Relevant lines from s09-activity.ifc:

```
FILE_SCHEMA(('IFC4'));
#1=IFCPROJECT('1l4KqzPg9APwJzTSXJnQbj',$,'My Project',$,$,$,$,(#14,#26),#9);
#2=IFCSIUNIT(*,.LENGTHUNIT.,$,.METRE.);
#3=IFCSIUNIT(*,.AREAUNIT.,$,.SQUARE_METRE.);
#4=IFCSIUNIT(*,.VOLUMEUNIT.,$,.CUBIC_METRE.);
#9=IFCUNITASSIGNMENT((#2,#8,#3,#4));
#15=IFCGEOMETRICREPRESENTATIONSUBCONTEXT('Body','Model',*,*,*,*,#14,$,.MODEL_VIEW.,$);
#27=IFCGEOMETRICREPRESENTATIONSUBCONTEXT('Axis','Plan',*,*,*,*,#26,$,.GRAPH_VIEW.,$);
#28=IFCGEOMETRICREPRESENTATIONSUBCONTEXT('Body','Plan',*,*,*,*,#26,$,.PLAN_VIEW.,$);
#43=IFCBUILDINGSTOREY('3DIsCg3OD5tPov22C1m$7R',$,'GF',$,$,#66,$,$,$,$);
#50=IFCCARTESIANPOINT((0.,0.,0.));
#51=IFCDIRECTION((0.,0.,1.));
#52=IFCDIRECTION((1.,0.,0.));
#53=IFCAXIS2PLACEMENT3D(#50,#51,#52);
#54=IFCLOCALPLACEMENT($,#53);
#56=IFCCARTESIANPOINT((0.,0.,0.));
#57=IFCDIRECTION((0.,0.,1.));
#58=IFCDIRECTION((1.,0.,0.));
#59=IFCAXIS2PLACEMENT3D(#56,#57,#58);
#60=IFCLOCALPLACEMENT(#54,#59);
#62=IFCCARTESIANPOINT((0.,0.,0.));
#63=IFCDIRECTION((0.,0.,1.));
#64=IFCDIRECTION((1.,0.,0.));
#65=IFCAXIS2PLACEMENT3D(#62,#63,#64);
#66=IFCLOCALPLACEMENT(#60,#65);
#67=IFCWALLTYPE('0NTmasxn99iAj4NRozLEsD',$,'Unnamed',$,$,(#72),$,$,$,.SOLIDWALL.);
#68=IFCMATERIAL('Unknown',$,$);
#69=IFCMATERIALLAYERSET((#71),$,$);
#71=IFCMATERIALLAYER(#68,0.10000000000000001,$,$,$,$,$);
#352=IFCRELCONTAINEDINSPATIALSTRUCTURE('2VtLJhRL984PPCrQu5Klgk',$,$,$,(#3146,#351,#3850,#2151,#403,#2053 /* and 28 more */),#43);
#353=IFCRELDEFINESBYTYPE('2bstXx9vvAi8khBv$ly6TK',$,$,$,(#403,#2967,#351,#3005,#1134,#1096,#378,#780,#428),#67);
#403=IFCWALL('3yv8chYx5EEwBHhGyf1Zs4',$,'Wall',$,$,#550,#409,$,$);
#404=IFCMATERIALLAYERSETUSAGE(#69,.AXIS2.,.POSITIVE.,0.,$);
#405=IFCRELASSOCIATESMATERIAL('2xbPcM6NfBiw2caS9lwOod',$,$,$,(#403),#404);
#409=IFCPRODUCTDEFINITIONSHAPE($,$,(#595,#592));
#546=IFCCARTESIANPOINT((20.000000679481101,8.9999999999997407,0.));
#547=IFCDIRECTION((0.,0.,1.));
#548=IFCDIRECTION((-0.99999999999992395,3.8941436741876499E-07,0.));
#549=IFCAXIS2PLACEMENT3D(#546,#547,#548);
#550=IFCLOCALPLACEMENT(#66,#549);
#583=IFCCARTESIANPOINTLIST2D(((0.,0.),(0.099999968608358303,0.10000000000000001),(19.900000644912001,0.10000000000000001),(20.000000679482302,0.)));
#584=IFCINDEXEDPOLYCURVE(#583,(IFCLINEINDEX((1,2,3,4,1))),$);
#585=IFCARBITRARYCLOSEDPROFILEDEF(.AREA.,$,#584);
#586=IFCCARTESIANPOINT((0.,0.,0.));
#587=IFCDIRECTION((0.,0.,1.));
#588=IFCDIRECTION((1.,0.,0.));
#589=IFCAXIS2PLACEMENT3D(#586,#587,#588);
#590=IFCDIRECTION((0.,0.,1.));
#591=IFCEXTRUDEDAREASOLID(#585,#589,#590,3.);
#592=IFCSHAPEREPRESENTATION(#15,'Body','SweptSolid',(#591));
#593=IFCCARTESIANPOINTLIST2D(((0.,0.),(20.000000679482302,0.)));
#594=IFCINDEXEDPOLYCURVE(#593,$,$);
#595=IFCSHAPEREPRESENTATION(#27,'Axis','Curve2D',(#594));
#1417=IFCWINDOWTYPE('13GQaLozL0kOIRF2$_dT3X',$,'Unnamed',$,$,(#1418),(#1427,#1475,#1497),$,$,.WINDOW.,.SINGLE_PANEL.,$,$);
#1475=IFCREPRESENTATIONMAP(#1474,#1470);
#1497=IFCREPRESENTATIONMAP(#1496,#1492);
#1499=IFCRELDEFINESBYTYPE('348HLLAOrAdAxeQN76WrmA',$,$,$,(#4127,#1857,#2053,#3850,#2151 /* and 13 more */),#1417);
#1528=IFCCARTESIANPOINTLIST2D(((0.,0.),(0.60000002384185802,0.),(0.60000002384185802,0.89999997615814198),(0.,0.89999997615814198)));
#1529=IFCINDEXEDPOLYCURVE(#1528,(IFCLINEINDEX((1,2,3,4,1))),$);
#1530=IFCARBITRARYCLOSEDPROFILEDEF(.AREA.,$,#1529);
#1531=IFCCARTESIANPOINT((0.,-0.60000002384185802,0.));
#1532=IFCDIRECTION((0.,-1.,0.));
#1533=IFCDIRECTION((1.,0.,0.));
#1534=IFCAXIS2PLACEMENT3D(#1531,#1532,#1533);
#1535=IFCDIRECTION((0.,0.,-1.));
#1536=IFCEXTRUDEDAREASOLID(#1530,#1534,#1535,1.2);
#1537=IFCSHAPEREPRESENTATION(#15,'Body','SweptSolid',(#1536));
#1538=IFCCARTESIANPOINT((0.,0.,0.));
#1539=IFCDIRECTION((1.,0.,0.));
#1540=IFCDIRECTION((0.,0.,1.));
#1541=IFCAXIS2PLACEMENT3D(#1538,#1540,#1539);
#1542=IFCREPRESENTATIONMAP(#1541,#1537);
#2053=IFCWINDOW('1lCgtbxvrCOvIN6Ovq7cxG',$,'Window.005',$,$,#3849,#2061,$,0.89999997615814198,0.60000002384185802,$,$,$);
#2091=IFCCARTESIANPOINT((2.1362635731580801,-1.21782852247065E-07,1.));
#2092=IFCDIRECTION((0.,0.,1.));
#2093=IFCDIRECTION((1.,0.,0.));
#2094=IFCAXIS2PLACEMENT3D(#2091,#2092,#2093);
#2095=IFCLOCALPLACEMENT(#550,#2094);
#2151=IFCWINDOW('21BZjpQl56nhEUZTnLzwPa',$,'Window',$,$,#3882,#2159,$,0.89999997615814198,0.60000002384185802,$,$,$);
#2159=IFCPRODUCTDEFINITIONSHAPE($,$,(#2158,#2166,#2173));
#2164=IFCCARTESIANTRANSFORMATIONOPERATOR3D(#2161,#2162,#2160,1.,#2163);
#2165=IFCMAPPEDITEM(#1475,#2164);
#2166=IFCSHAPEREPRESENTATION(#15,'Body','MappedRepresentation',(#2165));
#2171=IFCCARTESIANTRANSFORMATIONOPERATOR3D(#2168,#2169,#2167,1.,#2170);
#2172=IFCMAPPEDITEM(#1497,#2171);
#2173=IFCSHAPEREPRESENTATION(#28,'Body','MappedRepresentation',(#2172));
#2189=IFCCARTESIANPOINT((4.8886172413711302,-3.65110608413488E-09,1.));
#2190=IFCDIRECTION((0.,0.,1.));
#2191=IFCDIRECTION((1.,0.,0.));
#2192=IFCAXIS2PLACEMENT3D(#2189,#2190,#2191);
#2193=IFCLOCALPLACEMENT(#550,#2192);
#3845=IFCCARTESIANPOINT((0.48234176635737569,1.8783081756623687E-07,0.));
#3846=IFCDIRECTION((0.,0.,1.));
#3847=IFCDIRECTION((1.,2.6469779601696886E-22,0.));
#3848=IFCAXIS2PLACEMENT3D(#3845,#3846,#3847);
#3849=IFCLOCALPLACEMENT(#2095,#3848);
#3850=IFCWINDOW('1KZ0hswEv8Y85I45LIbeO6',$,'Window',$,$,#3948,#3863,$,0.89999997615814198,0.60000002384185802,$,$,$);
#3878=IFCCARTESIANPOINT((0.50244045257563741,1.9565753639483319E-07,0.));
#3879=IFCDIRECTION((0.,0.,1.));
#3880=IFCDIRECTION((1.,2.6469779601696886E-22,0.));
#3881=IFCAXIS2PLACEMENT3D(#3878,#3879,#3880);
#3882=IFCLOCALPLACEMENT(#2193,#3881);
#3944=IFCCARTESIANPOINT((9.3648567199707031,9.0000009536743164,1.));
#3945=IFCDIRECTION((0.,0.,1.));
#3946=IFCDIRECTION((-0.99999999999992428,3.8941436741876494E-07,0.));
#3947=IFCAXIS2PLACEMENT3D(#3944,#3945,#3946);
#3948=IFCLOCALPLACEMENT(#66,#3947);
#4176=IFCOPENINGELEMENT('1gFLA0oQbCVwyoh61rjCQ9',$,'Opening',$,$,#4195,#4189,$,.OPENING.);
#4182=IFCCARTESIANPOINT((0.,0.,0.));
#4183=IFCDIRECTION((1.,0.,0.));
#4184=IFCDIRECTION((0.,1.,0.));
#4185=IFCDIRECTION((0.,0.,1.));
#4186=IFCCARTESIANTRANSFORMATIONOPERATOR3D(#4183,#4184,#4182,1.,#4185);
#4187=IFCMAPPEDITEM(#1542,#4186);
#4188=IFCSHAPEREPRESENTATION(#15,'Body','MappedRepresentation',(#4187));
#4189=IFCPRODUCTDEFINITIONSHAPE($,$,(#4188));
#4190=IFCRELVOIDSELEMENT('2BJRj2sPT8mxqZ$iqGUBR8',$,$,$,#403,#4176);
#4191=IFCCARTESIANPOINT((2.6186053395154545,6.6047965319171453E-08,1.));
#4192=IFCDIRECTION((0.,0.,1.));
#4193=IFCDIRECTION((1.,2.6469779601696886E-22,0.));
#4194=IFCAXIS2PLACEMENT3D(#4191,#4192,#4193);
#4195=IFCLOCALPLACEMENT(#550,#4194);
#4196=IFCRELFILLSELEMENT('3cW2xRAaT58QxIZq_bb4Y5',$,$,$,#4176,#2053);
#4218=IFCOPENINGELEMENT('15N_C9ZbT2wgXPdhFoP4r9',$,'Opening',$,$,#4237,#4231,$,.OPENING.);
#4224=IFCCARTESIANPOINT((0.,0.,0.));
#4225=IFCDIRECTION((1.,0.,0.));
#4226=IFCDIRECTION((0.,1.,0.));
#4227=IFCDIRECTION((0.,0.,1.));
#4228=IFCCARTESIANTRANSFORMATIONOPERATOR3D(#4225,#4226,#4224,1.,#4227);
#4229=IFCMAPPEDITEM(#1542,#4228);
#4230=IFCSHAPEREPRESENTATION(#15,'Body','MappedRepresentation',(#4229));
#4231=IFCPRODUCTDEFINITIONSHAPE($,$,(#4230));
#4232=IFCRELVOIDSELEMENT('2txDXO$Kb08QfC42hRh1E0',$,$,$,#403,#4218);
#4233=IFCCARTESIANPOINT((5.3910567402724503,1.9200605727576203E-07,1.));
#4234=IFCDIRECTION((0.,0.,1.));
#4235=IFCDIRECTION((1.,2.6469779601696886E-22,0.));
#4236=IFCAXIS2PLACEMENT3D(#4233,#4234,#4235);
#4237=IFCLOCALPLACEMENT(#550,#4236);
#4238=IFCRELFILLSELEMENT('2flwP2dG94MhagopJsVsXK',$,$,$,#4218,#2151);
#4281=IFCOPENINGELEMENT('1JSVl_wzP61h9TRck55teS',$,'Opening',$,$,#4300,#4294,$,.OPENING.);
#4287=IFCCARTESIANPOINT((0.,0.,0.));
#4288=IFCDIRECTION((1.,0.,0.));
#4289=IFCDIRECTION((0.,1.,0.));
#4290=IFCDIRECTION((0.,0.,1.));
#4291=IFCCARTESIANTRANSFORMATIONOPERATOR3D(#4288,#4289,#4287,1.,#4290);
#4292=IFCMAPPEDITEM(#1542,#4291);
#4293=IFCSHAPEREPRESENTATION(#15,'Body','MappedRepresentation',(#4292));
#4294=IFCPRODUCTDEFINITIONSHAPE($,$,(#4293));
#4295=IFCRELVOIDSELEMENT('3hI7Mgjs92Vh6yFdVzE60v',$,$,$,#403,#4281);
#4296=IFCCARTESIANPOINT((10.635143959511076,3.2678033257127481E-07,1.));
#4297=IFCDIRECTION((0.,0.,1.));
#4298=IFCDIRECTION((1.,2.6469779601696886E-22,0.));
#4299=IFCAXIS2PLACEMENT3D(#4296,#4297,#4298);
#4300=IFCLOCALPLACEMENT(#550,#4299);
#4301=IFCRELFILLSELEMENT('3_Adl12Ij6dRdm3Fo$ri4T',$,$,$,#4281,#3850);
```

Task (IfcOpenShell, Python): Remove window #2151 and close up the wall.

```python
import ifcopenshell
import ifcopenshell.api.feature
import ifcopenshell.api.root
import ifcopenshell.geom
import ifcopenshell.util.shape

model = ifcopenshell.open("s09-activity.ifc")
settings = ifcopenshell.geom.settings()


def volume(element):
    """Net volume in cubic metres, openings subtracted."""
    shape = ifcopenshell.geom.create_shape(settings, element)
    return ifcopenshell.util.shape.get_volume(shape.geometry)


window = model.by_guid("21BZjpQl56nhEUZTnLzwPa")
opening = window.FillsVoids[0].RelatingOpeningElement
wall = opening.VoidsElements[0].RelatingBuildingElement
before = volume(wall)

ifcopenshell.api.root.remove_product(model, product=window)
ifcopenshell.api.feature.remove_feature(model, feature=opening)

after = volume(wall)

print(f"wall volume {before:.3f} -> {after:.3f} m3")

model.write("s09-activity_rev.ifc")
```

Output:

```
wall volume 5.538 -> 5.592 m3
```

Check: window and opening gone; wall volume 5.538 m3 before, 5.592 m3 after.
